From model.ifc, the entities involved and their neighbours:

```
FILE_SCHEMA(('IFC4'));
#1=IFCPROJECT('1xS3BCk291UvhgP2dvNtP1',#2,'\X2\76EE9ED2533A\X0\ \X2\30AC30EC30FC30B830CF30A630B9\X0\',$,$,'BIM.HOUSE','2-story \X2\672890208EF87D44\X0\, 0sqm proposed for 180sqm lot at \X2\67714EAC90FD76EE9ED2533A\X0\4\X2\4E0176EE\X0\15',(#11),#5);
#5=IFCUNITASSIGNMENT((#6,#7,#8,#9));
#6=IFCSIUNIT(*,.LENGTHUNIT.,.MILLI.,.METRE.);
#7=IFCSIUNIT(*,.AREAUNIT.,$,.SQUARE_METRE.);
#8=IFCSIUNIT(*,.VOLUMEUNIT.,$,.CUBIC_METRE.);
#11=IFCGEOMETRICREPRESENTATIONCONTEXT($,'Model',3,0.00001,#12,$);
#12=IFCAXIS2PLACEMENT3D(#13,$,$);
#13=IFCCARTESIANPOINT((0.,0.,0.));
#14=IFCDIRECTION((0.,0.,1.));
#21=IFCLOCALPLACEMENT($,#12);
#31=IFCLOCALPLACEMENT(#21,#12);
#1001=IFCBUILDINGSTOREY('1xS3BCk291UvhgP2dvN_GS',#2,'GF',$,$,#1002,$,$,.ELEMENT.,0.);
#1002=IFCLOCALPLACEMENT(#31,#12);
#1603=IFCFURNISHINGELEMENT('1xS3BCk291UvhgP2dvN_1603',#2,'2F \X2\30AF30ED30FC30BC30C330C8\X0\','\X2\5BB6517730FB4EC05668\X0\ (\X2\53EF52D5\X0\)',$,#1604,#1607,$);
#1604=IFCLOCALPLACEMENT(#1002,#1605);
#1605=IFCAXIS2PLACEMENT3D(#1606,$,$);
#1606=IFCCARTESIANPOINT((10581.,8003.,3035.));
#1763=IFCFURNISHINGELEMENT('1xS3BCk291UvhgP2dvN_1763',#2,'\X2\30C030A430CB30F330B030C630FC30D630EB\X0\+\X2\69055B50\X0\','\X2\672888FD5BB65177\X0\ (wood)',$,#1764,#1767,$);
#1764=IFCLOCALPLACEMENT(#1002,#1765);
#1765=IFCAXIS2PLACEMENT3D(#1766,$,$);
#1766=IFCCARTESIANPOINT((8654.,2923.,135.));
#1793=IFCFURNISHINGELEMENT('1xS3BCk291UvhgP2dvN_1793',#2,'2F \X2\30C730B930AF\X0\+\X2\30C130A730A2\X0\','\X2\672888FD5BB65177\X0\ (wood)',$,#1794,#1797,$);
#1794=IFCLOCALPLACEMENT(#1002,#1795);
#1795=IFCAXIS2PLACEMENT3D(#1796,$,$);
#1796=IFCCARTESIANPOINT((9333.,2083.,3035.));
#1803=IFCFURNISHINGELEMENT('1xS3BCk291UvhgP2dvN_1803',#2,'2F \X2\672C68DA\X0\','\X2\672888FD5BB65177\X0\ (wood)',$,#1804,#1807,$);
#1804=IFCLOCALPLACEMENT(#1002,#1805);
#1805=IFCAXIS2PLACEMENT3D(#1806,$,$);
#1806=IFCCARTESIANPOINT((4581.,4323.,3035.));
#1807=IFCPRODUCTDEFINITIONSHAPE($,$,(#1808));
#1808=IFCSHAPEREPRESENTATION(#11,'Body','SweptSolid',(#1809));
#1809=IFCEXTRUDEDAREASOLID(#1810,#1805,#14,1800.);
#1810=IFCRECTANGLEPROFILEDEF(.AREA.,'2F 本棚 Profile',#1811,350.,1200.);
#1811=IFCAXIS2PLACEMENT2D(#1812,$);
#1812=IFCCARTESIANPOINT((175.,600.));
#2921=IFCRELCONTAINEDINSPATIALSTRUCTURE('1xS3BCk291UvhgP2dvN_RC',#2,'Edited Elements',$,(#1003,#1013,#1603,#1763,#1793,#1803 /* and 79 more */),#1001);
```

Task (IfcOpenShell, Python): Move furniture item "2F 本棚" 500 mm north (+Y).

```python
import ifcopenshell
import ifcopenshell.api.geometry
import ifcopenshell.util.placement
import ifcopenshell.util.unit

model = ifcopenshell.open("model.ifc")
unit_scale = ifcopenshell.util.unit.calculate_unit_scale(model)

item = model.by_id(1803)
matrix = ifcopenshell.util.placement.get_local_placement(item.ObjectPlacement)
matrix[1, 3] += 0.5 / unit_scale
ifcopenshell.api.geometry.edit_object_placement(model, product=item, matrix=matrix, is_si=False)

print(ifcopenshell.util.placement.get_local_placement(item.ObjectPlacement).round(3) + 0.0)

model.write("model_updated.ifc")
```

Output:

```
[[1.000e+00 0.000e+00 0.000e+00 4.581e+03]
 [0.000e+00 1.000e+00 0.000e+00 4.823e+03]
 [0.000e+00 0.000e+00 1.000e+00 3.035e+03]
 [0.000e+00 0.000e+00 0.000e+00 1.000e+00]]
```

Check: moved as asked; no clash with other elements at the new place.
